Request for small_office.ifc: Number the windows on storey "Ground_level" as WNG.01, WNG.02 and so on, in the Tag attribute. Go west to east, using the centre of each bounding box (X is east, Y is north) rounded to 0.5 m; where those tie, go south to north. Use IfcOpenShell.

First a look at what the model holds.

```python
import ifcopenshell
import ifcopenshell.util.element
import ifcopenshell.util.placement

model = ifcopenshell.open("small_office.ifc")
print(model.schema)
storey = next(s for s in model.by_type("IfcBuildingStorey") if s.Name == "Ground_level")
windows = [e for e in ifcopenshell.util.element.get_decomposition(storey) if e.is_a("IfcWindow")]
for e in sorted(windows, key=lambda e: e.id()):
    origin = ifcopenshell.util.placement.get_local_placement(e.ObjectPlacement)[:3, 3]
    print(e.id(), e.Tag, e.Name, origin.round(2) + 0.0, sep=" | ")
```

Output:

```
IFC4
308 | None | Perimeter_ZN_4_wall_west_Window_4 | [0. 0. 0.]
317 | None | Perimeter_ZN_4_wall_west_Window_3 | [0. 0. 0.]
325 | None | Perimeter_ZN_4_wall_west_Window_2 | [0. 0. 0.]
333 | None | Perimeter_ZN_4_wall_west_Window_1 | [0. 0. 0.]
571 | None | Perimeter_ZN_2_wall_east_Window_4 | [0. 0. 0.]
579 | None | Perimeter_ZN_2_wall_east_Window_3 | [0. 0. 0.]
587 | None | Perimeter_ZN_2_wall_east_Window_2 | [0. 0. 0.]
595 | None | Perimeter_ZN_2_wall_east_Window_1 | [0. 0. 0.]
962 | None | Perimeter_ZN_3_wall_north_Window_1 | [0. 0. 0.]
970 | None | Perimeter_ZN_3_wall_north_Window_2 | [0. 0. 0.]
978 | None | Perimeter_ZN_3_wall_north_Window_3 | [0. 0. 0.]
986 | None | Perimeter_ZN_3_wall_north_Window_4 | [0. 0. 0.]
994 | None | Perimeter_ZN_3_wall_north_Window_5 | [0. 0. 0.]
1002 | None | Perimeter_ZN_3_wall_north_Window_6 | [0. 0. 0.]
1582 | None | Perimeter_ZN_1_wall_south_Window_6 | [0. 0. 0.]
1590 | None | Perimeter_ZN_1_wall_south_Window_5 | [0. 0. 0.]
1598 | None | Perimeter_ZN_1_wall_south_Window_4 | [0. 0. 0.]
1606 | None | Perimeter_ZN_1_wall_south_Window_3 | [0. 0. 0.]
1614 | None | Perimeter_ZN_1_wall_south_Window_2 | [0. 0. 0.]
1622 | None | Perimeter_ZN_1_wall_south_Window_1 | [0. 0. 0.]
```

```python
import ifcopenshell
import ifcopenshell.geom
import ifcopenshell.util.element
import ifcopenshell.util.shape

model = ifcopenshell.open("small_office.ifc")
settings = ifcopenshell.geom.settings()
settings.set("use-world-coords", True)


def centre(element):
    shape = ifcopenshell.geom.create_shape(settings, element)
    return ifcopenshell.util.shape.get_bbox_centroid(shape.geometry)


storey = next(s for s in model.by_type("IfcBuildingStorey") if s.Name == "Ground_level")
windows = [e for e in ifcopenshell.util.element.get_decomposition(storey) if e.is_a("IfcWindow")]

# Insertion points can sit at a corner or the storey origin, so sort by the geometry (in metres).
centres = {e: centre(e) for e in windows}
windows.sort(key=lambda e: (round(centres[e][0] / 0.5), centres[e][1]))

for i, e in enumerate(windows, start=1):
    number = f"WNG.{i:02d}"
    e.Tag = number
    print(e.id(), number)

model.write("small_office_edited.ifc")
```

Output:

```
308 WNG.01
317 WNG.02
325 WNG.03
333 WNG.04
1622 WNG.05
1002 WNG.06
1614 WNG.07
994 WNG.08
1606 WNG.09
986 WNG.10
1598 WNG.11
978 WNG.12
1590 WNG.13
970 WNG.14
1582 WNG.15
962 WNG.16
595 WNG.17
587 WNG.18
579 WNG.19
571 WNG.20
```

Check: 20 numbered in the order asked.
